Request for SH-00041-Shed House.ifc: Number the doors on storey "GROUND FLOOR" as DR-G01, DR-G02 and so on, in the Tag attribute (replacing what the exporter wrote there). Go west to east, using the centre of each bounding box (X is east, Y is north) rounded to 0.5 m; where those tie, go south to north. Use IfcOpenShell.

First a look at what the model holds.

```python
import ifcopenshell
import ifcopenshell.util.element
import ifcopenshell.util.placement

model = ifcopenshell.open("SH-00041-Shed House.ifc")
print(model.schema)
storey = next(s for s in model.by_type("IfcBuildingStorey") if s.Name == "GROUND FLOOR")
doors = [e for e in ifcopenshell.util.element.get_decomposition(storey) if e.is_a("IfcDoor")]
for e in sorted(doors, key=lambda e: e.id()):
    origin = ifcopenshell.util.placement.get_local_placement(e.ObjectPlacement)[:3, 3]
    print(e.id(), e.Tag, e.Name, origin.round(2) + 0.0, sep=" | ")
```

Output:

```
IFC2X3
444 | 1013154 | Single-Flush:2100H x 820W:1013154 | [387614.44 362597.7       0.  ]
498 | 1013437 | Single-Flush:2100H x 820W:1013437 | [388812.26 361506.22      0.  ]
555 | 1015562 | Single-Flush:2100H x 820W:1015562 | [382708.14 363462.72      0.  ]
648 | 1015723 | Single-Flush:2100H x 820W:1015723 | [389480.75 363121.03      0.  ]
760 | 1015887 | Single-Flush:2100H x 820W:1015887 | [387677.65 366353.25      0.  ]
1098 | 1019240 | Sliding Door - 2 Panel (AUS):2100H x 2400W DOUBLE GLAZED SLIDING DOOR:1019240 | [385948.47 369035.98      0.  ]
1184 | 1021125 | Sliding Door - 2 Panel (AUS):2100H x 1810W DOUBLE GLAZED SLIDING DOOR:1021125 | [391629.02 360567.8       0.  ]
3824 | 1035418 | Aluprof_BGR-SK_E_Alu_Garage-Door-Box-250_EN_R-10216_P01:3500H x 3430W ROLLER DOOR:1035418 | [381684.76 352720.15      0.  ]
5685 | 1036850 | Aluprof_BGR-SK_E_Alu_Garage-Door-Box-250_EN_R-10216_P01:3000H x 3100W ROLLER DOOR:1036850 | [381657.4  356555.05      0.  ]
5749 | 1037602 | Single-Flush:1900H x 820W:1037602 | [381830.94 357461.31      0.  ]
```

```python
import ifcopenshell
import ifcopenshell.geom
import ifcopenshell.util.element
import ifcopenshell.util.shape

model = ifcopenshell.open("SH-00041-Shed House.ifc")
settings = ifcopenshell.geom.settings()
settings.set("use-world-coords", True)


def centre(element):
    shape = ifcopenshell.geom.create_shape(settings, element)
    return ifcopenshell.util.shape.get_bbox_centroid(shape.geometry)


storey = next(s for s in model.by_type("IfcBuildingStorey") if s.Name == "GROUND FLOOR")
doors = [e for e in ifcopenshell.util.element.get_decomposition(storey) if e.is_a("IfcDoor")]

# Insertion points can sit at a corner or the storey origin, so sort by the geometry (in metres).
centres = {e: centre(e) for e in doors}
doors.sort(key=lambda e: (round(centres[e][0] / 0.5), centres[e][1]))

for i, e in enumerate(doors, start=1):
    number = f"DR-G{i:02d}"
    e.Tag = number
    print(e.id(), number)

model.write("SH-00041-Shed House-out.ifc")
```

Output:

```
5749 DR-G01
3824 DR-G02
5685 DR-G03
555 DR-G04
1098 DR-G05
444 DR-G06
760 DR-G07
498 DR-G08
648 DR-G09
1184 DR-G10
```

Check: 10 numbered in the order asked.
